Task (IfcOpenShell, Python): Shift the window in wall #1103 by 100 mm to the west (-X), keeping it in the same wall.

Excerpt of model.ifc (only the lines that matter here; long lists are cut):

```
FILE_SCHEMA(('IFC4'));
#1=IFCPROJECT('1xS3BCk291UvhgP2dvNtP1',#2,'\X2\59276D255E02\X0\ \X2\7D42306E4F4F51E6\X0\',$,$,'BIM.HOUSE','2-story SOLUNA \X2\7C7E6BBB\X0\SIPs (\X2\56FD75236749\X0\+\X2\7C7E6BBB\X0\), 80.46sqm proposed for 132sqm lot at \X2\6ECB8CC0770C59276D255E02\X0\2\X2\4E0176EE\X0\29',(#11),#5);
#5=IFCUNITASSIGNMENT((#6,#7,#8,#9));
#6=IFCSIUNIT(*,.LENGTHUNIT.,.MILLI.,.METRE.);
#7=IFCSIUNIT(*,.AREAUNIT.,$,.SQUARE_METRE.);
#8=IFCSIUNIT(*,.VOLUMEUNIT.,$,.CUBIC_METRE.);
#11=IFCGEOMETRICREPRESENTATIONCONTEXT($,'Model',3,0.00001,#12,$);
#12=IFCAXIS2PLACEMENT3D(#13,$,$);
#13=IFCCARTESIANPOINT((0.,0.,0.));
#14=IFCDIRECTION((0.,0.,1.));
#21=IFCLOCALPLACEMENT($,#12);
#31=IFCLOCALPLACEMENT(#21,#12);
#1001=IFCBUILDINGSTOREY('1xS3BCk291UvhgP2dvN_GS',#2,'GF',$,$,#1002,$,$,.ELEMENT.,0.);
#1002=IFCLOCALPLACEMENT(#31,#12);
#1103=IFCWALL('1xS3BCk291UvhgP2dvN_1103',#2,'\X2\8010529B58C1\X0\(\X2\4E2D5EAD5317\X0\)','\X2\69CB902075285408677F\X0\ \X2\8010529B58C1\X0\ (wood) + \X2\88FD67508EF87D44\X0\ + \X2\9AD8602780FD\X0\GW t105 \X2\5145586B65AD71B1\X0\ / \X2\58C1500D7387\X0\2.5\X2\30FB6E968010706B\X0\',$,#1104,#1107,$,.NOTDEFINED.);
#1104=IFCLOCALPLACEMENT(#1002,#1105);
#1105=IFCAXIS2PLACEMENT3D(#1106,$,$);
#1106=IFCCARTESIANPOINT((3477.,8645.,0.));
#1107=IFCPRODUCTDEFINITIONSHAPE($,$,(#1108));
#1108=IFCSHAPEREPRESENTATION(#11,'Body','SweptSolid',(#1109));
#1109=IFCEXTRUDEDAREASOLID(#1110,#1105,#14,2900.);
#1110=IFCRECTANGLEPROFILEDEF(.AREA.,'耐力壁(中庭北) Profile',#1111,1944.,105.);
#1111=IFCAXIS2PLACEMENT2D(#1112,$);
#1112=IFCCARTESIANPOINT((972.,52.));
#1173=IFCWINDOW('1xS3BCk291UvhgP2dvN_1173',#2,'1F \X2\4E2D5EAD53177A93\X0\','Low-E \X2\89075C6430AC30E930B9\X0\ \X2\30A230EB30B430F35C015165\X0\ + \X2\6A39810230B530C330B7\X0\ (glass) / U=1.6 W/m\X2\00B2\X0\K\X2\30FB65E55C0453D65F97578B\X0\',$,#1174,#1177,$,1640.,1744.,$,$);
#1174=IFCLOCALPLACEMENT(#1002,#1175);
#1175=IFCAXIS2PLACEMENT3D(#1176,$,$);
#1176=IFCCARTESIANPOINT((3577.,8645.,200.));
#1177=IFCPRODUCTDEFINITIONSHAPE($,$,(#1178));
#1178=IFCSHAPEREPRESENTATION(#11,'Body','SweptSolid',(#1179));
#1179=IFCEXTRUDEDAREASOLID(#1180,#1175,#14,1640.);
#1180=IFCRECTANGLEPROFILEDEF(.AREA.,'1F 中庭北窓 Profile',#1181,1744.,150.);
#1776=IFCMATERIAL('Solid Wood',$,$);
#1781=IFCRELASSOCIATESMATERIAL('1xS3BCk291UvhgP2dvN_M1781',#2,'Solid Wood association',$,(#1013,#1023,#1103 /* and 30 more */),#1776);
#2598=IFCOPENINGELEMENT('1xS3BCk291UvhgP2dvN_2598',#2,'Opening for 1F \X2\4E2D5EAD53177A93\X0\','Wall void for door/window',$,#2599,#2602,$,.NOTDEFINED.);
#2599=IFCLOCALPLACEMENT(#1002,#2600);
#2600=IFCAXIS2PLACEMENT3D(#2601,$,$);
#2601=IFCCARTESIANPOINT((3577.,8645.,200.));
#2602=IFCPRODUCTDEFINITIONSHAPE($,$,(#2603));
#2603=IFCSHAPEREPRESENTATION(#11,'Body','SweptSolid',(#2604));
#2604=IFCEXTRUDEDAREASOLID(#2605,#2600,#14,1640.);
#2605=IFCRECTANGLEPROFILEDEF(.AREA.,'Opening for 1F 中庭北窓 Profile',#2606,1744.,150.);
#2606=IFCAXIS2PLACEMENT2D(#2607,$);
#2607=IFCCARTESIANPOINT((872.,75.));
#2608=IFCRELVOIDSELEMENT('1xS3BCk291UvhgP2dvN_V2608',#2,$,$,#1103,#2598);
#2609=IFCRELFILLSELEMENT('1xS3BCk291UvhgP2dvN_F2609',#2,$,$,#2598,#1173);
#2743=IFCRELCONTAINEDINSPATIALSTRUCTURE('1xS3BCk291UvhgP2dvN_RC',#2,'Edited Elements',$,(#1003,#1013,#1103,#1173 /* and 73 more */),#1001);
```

```python
import ifcopenshell
import ifcopenshell.api.geometry
import ifcopenshell.util.placement

model = ifcopenshell.open("model.ifc")

window = model.by_guid("1xS3BCk291UvhgP2dvN_1173")
opening = window.FillsVoids[0].RelatingOpeningElement
wall = opening.VoidsElements[0].RelatingBuildingElement

wall_matrix = ifcopenshell.util.placement.get_local_placement(wall.ObjectPlacement)
shift = wall_matrix[:3, 0] * -100.0
before = ifcopenshell.util.placement.get_local_placement(window.ObjectPlacement)[:3, 3].copy()

# The window is not placed relative to its opening, so move both.
for product in (opening, window):
    matrix = ifcopenshell.util.placement.get_local_placement(product.ObjectPlacement)
    matrix[:3, 3] += shift
    ifcopenshell.api.geometry.edit_object_placement(model, product=product, matrix=matrix, is_si=False)

after = ifcopenshell.util.placement.get_local_placement(window.ObjectPlacement)[:3, 3]
print("window moved by", (after - before).round(3) + 0.0)

model.write("model_v2.ifc")
```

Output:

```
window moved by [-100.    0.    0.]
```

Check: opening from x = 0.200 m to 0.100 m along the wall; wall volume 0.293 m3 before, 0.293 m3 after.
